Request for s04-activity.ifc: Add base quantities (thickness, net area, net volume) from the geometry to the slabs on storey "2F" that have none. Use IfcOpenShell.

First a look at what the model holds.

```python
import ifcopenshell
import ifcopenshell.util.element
import ifcopenshell.util.unit

model = ifcopenshell.open("s04-activity.ifc")
print(model.schema)
for unit_type in ("LENGTHUNIT", "AREAUNIT", "VOLUMEUNIT"):
    print(unit_type, ifcopenshell.util.unit.calculate_unit_scale(model, unit_type))
storey = next(s for s in model.by_type("IfcBuildingStorey") if s.Name == "2F")
slabs = [e for e in ifcopenshell.util.element.get_decomposition(storey) if e.is_a("IfcSlab")]
for e in sorted(slabs, key=lambda e: e.id()):
    print(e.id(), e.is_a(), e.Name, list(ifcopenshell.util.element.get_psets(e, qtos_only=True)), sep=" | ")
```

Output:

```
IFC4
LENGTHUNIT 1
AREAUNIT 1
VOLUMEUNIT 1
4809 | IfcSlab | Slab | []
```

```python
import ifcopenshell
import ifcopenshell.api.pset
import ifcopenshell.geom
import ifcopenshell.util.element
import ifcopenshell.util.shape
import ifcopenshell.util.unit

model = ifcopenshell.open("s04-activity.ifc")
unit_scale = ifcopenshell.util.unit.calculate_unit_scale(model)
area_scale = ifcopenshell.util.unit.calculate_unit_scale(model, "AREAUNIT")
volume_scale = ifcopenshell.util.unit.calculate_unit_scale(model, "VOLUMEUNIT")
settings = ifcopenshell.geom.settings()

storey = next(s for s in model.by_type("IfcBuildingStorey") if s.Name == "2F")
slabs = [e for e in ifcopenshell.util.element.get_decomposition(storey) if e.is_a("IfcSlab")]

for e in sorted(slabs, key=lambda e: e.id()):
    if ifcopenshell.util.element.get_psets(e, qtos_only=True, should_inherit=False):
        continue
    # Geometry comes back in metres, in the element's own axes.
    shape = ifcopenshell.geom.create_shape(settings, e)
    values = {
        "Width": ifcopenshell.util.shape.get_z(shape.geometry) / unit_scale,
        "NetArea": ifcopenshell.util.shape.get_footprint_area(shape.geometry) / area_scale,
        "NetVolume": ifcopenshell.util.shape.get_volume(shape.geometry) / volume_scale,
    }
    qto = ifcopenshell.api.pset.add_qto(model, product=e, name="Qto_SlabBaseQuantities")
    ifcopenshell.api.pset.edit_qto(model, qto=qto, properties=values)
    print(e.id(), {k: round(v, 3) for k, v in values.items()})

model.write("s04-activity-out.ifc")
```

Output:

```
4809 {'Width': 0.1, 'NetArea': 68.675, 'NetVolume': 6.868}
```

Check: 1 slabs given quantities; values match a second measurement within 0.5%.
